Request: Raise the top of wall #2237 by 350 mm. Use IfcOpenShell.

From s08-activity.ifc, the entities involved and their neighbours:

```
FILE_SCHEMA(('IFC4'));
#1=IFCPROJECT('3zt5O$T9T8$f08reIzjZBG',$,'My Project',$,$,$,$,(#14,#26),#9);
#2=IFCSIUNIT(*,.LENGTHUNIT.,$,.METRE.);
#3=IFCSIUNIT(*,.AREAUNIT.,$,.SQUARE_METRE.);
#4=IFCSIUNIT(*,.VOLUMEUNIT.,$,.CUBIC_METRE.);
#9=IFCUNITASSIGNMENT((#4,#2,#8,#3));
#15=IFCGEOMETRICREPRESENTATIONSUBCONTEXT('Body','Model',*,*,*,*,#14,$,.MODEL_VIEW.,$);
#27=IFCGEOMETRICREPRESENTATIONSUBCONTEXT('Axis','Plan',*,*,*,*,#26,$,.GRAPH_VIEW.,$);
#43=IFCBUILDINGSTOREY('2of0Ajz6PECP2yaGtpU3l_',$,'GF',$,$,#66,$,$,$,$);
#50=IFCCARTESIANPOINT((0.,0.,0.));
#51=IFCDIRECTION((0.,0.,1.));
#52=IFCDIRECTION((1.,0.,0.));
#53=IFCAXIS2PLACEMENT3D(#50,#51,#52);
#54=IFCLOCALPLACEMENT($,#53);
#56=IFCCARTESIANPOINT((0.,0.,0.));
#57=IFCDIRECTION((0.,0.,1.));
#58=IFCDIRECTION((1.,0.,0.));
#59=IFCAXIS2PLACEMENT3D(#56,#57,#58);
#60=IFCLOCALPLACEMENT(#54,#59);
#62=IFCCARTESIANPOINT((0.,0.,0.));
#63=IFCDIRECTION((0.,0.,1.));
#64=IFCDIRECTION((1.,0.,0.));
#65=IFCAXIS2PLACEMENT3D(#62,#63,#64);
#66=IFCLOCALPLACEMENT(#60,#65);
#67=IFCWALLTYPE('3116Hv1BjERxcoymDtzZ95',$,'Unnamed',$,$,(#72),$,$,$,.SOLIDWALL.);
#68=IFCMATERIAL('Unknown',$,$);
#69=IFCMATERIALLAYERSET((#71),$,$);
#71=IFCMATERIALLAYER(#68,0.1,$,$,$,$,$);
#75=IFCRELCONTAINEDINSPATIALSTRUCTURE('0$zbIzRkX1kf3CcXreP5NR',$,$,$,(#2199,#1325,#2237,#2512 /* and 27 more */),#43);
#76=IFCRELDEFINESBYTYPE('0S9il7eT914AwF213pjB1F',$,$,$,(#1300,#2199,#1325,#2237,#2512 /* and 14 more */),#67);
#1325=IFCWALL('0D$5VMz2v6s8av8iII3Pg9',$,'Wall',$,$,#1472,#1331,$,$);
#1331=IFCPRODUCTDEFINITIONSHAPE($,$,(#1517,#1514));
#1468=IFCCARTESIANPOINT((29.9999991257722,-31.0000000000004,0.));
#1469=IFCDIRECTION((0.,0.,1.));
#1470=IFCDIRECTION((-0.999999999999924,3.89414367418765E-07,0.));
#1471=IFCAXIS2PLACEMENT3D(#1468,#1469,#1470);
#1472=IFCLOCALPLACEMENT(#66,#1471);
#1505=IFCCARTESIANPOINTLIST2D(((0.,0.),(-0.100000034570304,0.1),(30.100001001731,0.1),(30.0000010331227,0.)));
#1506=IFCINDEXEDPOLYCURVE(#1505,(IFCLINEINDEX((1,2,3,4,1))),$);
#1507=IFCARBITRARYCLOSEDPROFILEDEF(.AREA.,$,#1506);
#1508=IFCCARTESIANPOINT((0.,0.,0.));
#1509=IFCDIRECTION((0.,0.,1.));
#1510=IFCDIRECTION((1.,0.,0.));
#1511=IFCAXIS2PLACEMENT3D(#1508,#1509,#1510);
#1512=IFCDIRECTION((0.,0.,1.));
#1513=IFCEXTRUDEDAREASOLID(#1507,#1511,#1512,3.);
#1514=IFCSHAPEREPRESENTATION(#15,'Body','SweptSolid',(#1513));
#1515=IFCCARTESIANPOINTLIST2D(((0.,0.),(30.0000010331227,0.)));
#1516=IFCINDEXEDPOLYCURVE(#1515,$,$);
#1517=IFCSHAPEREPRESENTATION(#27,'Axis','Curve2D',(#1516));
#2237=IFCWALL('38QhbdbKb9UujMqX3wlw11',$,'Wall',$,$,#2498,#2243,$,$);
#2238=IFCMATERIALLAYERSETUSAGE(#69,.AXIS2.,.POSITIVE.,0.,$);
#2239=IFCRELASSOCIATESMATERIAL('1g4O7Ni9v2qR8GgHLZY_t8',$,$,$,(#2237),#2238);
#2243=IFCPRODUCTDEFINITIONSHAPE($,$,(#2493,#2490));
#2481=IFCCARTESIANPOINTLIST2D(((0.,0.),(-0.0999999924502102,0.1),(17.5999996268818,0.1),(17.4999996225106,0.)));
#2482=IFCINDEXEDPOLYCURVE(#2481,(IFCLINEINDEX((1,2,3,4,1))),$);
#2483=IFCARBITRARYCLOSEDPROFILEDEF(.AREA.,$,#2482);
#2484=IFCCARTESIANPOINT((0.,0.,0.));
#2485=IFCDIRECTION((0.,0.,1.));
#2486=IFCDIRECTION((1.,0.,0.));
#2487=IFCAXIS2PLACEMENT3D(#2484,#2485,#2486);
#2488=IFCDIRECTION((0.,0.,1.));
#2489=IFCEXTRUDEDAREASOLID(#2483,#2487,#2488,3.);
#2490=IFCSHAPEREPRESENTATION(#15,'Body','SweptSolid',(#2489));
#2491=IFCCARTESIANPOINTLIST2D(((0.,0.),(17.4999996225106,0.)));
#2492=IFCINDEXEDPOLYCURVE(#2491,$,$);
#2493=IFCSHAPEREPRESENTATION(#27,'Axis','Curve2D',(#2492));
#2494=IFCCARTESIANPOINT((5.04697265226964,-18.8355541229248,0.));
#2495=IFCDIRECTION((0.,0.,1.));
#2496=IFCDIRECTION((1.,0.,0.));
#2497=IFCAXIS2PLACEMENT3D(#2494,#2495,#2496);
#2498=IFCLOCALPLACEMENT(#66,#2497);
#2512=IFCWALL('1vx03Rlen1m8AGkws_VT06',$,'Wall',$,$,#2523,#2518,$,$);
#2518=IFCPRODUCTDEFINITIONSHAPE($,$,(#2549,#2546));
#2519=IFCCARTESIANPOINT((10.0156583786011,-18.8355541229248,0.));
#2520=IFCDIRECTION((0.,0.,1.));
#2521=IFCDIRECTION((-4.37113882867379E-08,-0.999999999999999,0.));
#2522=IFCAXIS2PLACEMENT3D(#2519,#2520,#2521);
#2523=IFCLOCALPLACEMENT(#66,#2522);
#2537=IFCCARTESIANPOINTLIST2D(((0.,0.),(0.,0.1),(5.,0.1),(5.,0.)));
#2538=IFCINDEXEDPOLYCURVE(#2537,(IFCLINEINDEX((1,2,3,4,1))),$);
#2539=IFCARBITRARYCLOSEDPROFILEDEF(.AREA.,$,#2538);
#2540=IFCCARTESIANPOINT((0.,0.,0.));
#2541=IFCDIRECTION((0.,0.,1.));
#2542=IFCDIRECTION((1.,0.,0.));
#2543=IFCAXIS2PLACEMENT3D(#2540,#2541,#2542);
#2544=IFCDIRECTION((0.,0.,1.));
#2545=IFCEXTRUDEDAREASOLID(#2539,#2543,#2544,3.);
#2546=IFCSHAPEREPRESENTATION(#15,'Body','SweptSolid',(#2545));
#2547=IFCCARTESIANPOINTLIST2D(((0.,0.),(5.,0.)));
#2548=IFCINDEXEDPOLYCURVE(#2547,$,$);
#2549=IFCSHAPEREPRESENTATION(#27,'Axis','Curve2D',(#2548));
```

```python
import ifcopenshell
import ifcopenshell.geom
import ifcopenshell.util.representation
import ifcopenshell.util.shape
import ifcopenshell.util.unit

model = ifcopenshell.open("s08-activity.ifc")
unit_scale = ifcopenshell.util.unit.calculate_unit_scale(model)
settings = ifcopenshell.geom.settings()


def volume(element):
    """Net volume in cubic metres, openings subtracted."""
    shape = ifcopenshell.geom.create_shape(settings, element)
    return ifcopenshell.util.shape.get_volume(shape.geometry)


wall = model.by_id(2237)
before = volume(wall)

body = ifcopenshell.util.representation.get_representation(wall, "Model", "Body")
solid = body.Items[0]
old_height = solid.Depth
solid.Depth += 0.35 / unit_scale
after = volume(wall)

print(f"height {old_height:g} -> {solid.Depth:g}, volume {before:.3f} -> {after:.3f} m3")

model.write("s08-activity_updated.ifc")
```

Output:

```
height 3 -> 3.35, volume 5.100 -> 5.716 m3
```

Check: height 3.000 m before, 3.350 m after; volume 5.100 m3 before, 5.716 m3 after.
